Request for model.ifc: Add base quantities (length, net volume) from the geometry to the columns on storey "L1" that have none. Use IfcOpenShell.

First a look at what the model holds.

```python
import ifcopenshell
import ifcopenshell.util.element
import ifcopenshell.util.unit

model = ifcopenshell.open("model.ifc")
print(model.schema)
for unit_type in ("LENGTHUNIT", "AREAUNIT", "VOLUMEUNIT"):
    print(unit_type, ifcopenshell.util.unit.calculate_unit_scale(model, unit_type))
storey = next(s for s in model.by_type("IfcBuildingStorey") if s.Name == "L1")
columns = [e for e in ifcopenshell.util.element.get_decomposition(storey) if e.is_a("IfcColumn")]
for e in sorted(columns, key=lambda e: e.id()):
    print(e.id(), e.is_a(), e.Name, list(ifcopenshell.util.element.get_psets(e, qtos_only=True)), sep=" | ")
```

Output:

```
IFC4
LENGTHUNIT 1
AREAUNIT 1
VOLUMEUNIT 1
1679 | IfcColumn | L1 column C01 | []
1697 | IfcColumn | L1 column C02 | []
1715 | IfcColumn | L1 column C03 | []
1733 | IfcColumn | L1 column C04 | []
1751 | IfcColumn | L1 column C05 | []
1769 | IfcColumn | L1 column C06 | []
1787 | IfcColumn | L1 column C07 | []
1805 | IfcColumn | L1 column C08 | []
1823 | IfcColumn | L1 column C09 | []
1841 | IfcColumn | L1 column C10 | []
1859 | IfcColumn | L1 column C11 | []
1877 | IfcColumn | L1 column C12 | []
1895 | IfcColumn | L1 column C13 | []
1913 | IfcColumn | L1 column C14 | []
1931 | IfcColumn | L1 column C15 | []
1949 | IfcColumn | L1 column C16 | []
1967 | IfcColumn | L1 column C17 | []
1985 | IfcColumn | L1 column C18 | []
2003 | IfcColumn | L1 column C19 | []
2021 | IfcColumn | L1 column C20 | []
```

```python
import ifcopenshell
import ifcopenshell.api.pset
import ifcopenshell.geom
import ifcopenshell.util.element
import ifcopenshell.util.shape
import ifcopenshell.util.unit

model = ifcopenshell.open("model.ifc")
unit_scale = ifcopenshell.util.unit.calculate_unit_scale(model)
volume_scale = ifcopenshell.util.unit.calculate_unit_scale(model, "VOLUMEUNIT")
settings = ifcopenshell.geom.settings()

storey = next(s for s in model.by_type("IfcBuildingStorey") if s.Name == "L1")
columns = [e for e in ifcopenshell.util.element.get_decomposition(storey) if e.is_a("IfcColumn")]

for e in sorted(columns, key=lambda e: e.id()):
    if ifcopenshell.util.element.get_psets(e, qtos_only=True, should_inherit=False):
        continue
    # Geometry comes back in metres, in the element's own axes.
    shape = ifcopenshell.geom.create_shape(settings, e)
    values = {
        "Length": ifcopenshell.util.shape.get_z(shape.geometry) / unit_scale,
        "NetVolume": ifcopenshell.util.shape.get_volume(shape.geometry) / volume_scale,
    }
    qto = ifcopenshell.api.pset.add_qto(model, product=e, name="Qto_ColumnBaseQuantities")
    ifcopenshell.api.pset.edit_qto(model, qto=qto, properties=values)
    print(e.id(), {k: round(v, 3) for k, v in values.items()})

model.write("model_edited.ifc")
```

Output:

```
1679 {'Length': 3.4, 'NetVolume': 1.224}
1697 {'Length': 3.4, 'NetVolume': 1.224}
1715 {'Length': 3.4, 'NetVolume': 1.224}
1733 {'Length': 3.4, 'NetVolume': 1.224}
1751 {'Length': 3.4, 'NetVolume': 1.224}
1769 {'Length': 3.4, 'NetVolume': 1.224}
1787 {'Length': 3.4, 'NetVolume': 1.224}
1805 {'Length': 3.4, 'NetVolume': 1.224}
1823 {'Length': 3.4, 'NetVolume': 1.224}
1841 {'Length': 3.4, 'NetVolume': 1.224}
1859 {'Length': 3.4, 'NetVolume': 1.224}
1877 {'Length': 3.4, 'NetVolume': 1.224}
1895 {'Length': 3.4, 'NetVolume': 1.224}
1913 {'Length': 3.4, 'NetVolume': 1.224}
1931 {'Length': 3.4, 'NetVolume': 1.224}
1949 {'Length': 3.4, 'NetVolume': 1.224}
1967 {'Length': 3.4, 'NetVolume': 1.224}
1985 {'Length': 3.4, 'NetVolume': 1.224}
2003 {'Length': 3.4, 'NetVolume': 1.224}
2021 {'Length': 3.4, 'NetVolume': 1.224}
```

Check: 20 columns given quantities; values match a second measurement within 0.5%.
